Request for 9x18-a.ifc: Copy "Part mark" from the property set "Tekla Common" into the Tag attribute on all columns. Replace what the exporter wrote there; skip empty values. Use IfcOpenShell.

First a look at what the model holds.

```python
import ifcopenshell
import ifcopenshell.util.element

model = ifcopenshell.open("9x18-a.ifc")
print(model.schema)
columns = model.by_type("IfcColumn")
print(len(columns), "columns")
for e in columns[:8]:
    source = ifcopenshell.util.element.get_pset(e, "Tekla Common", "Part mark")
    target = e.Tag
    print(e.id(), repr(source), repr(target), sep=" | ")
```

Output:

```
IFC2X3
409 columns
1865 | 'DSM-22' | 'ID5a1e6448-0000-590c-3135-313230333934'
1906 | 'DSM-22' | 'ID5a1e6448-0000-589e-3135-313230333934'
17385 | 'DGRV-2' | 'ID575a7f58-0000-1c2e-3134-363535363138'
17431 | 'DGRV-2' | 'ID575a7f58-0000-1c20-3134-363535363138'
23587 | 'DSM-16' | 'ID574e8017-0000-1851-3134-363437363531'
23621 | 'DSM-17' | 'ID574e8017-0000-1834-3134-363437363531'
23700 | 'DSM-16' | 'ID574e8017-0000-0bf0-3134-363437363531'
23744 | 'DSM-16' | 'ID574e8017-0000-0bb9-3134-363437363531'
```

```python
import ifcopenshell
import ifcopenshell.util.element

model = ifcopenshell.open("9x18-a.ifc")

count = 0
for e in model.by_type("IfcColumn"):
    value = ifcopenshell.util.element.get_pset(e, "Tekla Common", "Part mark")
    current = e.Tag
    if not value or not value.strip() or current == value:
        continue
    e.Tag = value
    count += 1

print(count, "columns updated")

model.write("9x18-a_rev.ifc")
```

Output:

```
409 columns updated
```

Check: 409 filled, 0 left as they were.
